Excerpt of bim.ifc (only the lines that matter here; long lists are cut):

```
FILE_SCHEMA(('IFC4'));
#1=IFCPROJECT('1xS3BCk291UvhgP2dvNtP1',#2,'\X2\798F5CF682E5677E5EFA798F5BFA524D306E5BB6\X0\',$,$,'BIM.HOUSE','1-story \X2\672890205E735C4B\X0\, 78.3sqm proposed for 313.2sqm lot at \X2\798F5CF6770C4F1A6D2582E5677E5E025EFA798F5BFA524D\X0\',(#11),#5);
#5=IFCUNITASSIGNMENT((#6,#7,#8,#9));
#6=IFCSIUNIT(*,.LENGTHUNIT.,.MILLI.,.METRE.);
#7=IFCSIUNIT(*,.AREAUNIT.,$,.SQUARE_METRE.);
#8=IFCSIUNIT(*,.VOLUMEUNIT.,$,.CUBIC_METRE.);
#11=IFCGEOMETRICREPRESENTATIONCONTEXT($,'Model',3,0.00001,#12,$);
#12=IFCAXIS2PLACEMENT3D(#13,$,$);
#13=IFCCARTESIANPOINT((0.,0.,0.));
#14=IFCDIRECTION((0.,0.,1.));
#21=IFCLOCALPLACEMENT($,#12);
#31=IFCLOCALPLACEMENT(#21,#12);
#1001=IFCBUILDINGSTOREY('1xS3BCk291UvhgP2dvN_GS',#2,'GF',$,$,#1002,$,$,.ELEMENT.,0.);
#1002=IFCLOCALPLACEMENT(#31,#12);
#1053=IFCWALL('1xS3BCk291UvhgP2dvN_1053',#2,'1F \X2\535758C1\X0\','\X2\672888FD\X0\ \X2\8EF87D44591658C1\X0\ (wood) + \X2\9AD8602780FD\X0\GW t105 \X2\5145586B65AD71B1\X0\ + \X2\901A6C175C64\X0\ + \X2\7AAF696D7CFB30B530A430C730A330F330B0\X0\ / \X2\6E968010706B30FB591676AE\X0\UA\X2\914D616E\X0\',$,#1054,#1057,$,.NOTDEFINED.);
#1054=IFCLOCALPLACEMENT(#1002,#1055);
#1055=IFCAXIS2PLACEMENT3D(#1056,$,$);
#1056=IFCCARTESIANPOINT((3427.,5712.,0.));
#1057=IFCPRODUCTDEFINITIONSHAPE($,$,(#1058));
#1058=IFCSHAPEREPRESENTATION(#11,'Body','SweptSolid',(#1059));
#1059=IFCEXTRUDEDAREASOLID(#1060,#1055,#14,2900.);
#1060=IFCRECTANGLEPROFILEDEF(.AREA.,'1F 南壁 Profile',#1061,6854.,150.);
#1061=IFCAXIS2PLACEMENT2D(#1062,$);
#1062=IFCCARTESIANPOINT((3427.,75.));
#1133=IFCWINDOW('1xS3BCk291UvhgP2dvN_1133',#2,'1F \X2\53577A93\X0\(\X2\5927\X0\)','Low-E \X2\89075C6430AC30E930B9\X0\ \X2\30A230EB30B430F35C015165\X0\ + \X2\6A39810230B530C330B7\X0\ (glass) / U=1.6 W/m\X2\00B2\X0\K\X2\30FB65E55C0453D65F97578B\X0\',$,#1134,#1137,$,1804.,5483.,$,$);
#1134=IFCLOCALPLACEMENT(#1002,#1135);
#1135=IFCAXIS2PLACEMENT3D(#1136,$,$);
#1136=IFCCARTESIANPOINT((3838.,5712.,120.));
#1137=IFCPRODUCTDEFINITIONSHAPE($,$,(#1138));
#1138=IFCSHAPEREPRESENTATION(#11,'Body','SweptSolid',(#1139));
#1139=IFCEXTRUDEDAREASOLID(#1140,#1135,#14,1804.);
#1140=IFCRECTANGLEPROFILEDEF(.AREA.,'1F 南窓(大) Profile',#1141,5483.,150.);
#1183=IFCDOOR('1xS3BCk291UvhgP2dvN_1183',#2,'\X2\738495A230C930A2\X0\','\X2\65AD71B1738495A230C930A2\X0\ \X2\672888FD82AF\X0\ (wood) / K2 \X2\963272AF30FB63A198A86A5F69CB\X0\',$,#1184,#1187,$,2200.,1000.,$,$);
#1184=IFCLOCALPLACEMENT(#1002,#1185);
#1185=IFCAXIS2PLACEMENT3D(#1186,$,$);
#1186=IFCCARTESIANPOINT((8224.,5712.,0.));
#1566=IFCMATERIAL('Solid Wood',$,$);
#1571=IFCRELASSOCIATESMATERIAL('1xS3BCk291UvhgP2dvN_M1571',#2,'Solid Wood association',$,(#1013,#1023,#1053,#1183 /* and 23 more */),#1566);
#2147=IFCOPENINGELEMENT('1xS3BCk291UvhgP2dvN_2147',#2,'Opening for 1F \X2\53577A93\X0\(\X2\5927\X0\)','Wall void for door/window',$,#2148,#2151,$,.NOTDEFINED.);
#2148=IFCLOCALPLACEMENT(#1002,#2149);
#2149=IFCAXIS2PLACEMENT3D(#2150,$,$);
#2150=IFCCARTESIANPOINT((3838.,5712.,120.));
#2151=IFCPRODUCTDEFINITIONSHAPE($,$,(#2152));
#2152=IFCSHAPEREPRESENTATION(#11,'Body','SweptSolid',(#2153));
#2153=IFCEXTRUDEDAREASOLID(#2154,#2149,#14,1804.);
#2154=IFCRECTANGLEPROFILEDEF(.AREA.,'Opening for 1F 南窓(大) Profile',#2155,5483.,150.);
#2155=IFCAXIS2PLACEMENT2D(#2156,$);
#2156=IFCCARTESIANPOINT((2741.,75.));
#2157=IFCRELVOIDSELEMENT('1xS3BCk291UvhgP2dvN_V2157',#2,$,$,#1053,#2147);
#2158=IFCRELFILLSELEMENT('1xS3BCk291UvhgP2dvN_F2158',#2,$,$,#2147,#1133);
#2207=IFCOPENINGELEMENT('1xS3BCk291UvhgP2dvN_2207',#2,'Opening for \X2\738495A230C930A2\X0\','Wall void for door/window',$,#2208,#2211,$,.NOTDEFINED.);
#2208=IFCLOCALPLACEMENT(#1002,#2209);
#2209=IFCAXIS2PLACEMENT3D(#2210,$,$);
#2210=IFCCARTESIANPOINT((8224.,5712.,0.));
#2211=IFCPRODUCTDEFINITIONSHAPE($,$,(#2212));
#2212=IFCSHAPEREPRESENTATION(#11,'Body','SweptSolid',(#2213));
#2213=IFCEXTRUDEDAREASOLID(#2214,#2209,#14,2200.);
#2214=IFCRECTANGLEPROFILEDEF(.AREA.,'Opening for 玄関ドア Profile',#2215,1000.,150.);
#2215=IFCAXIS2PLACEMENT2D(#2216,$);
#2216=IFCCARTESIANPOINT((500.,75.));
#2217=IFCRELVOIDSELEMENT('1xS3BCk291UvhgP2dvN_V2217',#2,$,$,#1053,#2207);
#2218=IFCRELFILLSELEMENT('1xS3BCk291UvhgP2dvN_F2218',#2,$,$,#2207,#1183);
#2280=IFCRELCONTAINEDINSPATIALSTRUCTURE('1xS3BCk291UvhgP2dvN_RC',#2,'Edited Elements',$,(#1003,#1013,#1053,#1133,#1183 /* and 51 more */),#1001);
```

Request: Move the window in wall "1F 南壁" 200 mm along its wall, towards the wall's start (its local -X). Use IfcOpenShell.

```python
import ifcopenshell
import ifcopenshell.api.geometry
import ifcopenshell.util.placement
import ifcopenshell.util.unit

model = ifcopenshell.open("bim.ifc")
unit_scale = ifcopenshell.util.unit.calculate_unit_scale(model)

window = model.by_guid("1xS3BCk291UvhgP2dvN_1133")
opening = window.FillsVoids[0].RelatingOpeningElement
wall = opening.VoidsElements[0].RelatingBuildingElement

wall_matrix = ifcopenshell.util.placement.get_local_placement(wall.ObjectPlacement)
shift = wall_matrix[:3, 0] * -0.2 / unit_scale
before = ifcopenshell.util.placement.get_local_placement(window.ObjectPlacement)[:3, 3].copy()

# The window is not placed relative to its opening, so move both.
for product in (opening, window):
    matrix = ifcopenshell.util.placement.get_local_placement(product.ObjectPlacement)
    matrix[:3, 3] += shift
    ifcopenshell.api.geometry.edit_object_placement(model, product=product, matrix=matrix, is_si=False)

after = ifcopenshell.util.placement.get_local_placement(window.ObjectPlacement)[:3, 3]
print("window moved by", (after - before).round(3) + 0.0)

model.write("bim-out.ifc")
```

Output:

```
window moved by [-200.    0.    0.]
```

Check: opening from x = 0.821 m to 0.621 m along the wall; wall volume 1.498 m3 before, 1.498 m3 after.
